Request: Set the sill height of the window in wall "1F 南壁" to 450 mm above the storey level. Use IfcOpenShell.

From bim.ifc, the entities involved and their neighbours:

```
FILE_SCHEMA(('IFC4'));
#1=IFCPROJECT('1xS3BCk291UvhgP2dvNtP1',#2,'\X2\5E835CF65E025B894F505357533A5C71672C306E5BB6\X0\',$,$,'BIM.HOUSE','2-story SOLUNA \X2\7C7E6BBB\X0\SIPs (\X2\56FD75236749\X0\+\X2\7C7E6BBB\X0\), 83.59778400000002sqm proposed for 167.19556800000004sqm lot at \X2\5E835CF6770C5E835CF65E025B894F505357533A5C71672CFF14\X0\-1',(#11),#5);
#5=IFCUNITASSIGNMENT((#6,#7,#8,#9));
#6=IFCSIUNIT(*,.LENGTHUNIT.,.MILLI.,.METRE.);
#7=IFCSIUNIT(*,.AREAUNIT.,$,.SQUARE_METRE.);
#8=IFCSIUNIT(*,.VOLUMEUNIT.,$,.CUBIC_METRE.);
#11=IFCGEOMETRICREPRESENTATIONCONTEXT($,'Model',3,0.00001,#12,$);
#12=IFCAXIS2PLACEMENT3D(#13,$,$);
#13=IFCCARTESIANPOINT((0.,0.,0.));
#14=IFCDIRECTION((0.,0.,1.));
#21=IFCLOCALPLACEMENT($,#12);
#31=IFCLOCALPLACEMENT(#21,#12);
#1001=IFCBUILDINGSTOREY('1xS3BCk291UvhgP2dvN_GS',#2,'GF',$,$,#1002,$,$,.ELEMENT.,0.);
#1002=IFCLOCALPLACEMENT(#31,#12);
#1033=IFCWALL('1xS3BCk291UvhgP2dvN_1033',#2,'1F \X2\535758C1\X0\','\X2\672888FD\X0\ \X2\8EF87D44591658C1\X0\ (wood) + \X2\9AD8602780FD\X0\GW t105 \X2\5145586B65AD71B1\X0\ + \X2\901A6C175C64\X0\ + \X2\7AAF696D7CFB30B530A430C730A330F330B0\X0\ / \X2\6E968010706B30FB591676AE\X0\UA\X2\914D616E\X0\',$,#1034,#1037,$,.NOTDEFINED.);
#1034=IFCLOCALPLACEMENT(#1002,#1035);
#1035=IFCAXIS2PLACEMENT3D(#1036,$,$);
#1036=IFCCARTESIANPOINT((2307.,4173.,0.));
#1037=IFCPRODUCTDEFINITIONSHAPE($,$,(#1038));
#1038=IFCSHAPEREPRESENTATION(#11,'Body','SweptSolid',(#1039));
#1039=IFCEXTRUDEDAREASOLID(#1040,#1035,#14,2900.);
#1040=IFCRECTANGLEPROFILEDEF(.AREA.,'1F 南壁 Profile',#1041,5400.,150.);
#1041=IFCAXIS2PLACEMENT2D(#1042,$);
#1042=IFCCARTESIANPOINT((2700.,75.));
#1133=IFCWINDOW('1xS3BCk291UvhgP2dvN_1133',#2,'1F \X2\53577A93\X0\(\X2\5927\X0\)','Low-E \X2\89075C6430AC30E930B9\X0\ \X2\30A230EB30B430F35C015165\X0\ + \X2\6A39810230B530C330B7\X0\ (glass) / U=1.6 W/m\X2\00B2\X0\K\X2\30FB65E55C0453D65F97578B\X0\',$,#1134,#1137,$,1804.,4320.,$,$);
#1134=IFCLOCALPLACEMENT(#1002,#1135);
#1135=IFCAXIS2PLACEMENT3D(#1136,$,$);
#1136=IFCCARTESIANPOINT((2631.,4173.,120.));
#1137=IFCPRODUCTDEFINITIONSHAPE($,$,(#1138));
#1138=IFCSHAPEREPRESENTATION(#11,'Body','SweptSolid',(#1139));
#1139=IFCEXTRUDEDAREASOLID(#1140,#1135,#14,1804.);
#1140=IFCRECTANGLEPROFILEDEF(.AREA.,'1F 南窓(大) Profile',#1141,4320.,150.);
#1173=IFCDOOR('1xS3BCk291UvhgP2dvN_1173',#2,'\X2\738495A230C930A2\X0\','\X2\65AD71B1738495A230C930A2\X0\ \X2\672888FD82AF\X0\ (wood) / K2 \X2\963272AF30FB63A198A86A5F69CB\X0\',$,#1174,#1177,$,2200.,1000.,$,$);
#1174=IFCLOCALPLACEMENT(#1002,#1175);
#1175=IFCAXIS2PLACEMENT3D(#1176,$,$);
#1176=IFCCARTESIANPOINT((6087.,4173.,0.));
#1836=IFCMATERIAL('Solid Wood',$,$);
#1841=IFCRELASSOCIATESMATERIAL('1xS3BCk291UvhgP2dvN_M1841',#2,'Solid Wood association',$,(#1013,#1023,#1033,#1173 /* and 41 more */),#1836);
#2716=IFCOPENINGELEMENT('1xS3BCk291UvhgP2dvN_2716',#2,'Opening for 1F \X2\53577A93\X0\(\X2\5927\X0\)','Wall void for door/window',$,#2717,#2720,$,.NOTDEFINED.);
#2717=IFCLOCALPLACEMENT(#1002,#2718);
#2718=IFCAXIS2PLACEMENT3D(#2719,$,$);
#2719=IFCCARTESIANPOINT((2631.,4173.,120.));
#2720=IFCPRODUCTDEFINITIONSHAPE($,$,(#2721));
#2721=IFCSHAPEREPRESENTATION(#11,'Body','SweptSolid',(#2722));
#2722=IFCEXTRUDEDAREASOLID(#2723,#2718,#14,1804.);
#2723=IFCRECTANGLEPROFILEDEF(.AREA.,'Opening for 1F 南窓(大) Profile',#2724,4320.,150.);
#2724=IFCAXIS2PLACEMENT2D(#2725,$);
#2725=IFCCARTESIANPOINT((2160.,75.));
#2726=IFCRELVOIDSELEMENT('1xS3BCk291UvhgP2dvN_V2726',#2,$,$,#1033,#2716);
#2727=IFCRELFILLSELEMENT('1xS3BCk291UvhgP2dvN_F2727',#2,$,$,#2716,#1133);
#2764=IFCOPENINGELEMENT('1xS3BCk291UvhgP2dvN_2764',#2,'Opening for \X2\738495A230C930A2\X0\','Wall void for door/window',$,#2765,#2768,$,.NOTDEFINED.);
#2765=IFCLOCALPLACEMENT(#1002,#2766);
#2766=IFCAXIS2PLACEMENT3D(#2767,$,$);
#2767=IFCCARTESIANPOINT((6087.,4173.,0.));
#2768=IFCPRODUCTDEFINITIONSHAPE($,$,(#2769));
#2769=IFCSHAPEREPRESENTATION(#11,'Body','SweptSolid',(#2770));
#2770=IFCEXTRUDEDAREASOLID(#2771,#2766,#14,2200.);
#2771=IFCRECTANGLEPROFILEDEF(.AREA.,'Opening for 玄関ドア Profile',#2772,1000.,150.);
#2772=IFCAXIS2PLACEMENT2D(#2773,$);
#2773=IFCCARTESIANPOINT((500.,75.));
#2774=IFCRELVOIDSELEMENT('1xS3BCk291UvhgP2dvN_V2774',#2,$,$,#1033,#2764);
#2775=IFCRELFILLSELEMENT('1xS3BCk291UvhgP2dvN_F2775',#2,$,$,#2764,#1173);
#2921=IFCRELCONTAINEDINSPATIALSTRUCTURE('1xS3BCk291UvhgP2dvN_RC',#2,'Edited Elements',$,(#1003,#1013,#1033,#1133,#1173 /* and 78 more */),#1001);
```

```python
import numpy as np
import ifcopenshell
import ifcopenshell.api.geometry
import ifcopenshell.geom
import ifcopenshell.util.element
import ifcopenshell.util.placement
import ifcopenshell.util.shape
import ifcopenshell.util.unit

model = ifcopenshell.open("bim.ifc")
unit_scale = ifcopenshell.util.unit.calculate_unit_scale(model)

window = model.by_guid("1xS3BCk291UvhgP2dvN_1133")
opening = window.FillsVoids[0].RelatingOpeningElement
storey = ifcopenshell.util.element.get_container(window, ifc_class="IfcBuildingStorey")
level = ifcopenshell.util.placement.get_local_placement(storey.ObjectPlacement)[2, 3]

# The opening's origin need not be at the sill, so measure its lowest point.
shape = ifcopenshell.geom.create_shape(ifcopenshell.geom.settings(), opening)
bottom = ifcopenshell.util.shape.get_shape_bottom_elevation(shape, shape.geometry) / unit_scale
dz = level + 0.45 / unit_scale - bottom

shift = np.array([0.0, 0.0, dz])
# The window is not placed relative to its opening, so move both.
for product in (opening, window):
    matrix = ifcopenshell.util.placement.get_local_placement(product.ObjectPlacement)
    matrix[:3, 3] += shift
    ifcopenshell.api.geometry.edit_object_placement(model, product=product, matrix=matrix, is_si=False)

print(f"moved by {dz * unit_scale:+.3f} m")

model.write("bim-out.ifc")
```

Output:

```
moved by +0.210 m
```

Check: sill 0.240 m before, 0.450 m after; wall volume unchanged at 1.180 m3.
